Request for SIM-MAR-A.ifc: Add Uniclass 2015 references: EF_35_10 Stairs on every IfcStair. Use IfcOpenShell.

First a look at what the model holds.

```python
import ifcopenshell

model = ifcopenshell.open("SIM-MAR-A.ifc")
print(model.schema)
print("classifications:", [c.Name for c in model.by_type("IfcClassification")])
for ifc_class in ("IfcDoor", "IfcRoof", "IfcStair", "IfcWall", "IfcWindow"):
    print(ifc_class, len(model.by_type(ifc_class)))
```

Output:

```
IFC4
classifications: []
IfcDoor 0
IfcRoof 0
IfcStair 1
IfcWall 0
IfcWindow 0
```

```python
import ifcopenshell
import ifcopenshell.api.classification

model = ifcopenshell.open("SIM-MAR-A.ifc")

system = ifcopenshell.api.classification.add_classification(model, classification="Uniclass 2015")

codes = {
    "IfcStair": ("EF_35_10", "Stairs"),
}
for ifc_class, (code, name) in codes.items():
    products = model.by_type(ifc_class)
    ifcopenshell.api.classification.add_reference(
        model, products=products, classification=system, identification=code, name=name
    )
    print(code, len(products))

model.write("SIM-MAR-A_rev.ifc")
```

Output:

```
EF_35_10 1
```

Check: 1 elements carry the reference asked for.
